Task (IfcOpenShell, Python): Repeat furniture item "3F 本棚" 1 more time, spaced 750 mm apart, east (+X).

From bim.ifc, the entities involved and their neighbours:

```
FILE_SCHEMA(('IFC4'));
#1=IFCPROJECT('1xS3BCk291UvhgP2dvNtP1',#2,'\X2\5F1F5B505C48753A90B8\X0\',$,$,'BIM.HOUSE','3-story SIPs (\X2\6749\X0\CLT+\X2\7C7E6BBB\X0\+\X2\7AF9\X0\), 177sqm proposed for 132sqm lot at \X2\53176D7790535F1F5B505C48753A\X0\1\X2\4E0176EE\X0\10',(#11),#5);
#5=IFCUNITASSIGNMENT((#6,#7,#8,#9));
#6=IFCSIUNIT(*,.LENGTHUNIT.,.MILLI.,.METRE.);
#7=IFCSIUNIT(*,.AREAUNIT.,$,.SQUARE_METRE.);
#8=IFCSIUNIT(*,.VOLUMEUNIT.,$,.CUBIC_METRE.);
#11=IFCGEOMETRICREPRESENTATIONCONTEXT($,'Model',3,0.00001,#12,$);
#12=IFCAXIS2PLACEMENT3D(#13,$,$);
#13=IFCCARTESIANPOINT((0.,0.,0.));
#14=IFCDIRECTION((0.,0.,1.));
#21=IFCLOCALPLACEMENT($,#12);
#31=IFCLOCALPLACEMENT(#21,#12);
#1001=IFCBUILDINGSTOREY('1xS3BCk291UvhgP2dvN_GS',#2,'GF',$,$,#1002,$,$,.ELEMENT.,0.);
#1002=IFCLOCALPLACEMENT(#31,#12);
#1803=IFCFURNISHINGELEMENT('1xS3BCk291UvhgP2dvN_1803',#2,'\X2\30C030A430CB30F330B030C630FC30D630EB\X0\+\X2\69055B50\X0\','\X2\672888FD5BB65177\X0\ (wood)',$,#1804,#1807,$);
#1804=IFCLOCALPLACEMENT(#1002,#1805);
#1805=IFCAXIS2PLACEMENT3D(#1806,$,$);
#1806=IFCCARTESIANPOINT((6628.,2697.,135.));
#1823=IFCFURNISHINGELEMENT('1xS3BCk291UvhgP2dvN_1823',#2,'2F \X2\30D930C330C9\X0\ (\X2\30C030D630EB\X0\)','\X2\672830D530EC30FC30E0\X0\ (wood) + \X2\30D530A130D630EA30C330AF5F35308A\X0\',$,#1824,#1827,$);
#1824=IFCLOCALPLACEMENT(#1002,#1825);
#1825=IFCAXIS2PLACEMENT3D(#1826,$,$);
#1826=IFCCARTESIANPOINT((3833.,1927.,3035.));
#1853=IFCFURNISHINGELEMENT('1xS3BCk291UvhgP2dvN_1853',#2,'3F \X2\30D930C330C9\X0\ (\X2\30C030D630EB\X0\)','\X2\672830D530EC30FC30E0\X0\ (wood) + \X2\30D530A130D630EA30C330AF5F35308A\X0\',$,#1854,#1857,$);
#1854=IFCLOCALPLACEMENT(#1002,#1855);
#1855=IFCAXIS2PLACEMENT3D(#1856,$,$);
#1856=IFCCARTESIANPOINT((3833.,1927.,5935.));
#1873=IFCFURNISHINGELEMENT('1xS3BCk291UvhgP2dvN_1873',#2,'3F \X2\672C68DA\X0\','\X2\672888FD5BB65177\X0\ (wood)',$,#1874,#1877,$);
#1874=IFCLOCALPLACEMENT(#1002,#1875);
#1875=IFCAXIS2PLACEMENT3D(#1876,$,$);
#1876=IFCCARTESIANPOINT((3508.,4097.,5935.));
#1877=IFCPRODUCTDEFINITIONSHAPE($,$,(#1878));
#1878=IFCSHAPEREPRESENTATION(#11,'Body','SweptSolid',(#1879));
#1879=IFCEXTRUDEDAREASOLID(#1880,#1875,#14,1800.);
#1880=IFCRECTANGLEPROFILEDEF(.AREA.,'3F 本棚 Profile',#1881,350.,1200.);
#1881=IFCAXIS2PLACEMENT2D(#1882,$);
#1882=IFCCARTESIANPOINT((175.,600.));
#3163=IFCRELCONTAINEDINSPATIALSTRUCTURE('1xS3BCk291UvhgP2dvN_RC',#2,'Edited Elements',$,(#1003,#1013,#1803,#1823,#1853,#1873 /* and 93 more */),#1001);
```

```python
import numpy as np
import ifcopenshell
import ifcopenshell.api.geometry
import ifcopenshell.api.root
import ifcopenshell.util.element
import ifcopenshell.util.placement
import ifcopenshell.util.unit

model = ifcopenshell.open("bim.ifc")
unit_scale = ifcopenshell.util.unit.calculate_unit_scale(model)


def reuse_history(source, copy):
    """copy_class also copies each property set's owner history, people and application; keep the originals."""
    for rel in copy.IsDefinedBy:
        if rel.is_a("IfcRelDefinesByProperties") and (history := rel.RelatingPropertyDefinition.OwnerHistory):
            rel.RelatingPropertyDefinition.OwnerHistory = source.OwnerHistory
            ifcopenshell.util.element.remove_deep2(model, history)


source = model.by_guid("1xS3BCk291UvhgP2dvN_1873")
base = ifcopenshell.util.placement.get_local_placement(source.ObjectPlacement)
step = np.array([1.0, 0.0, 0.0]) * 0.75 / unit_scale

for i in range(1, 2):
    copy = ifcopenshell.api.root.copy_class(model, product=source)
    copy.Representation = ifcopenshell.util.element.copy_deep(
        model, source.Representation, exclude=["IfcGeometricRepresentationContext", "IfcRepresentationMap"]
    )
    reuse_history(source, copy)
    matrix = base.copy()
    matrix[:3, 3] += i * step
    print("added at", matrix[:3, 3].round(3) + 0.0)
    ifcopenshell.api.geometry.edit_object_placement(model, product=copy, matrix=matrix, is_si=False)

model.write("bim_v2.ifc")
```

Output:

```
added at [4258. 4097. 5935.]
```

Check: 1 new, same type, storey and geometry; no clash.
